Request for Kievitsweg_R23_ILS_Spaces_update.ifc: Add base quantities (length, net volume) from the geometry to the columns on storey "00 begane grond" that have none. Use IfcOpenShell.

First a look at what the model holds.

```python
import ifcopenshell
import ifcopenshell.util.element
import ifcopenshell.util.unit

model = ifcopenshell.open("Kievitsweg_R23_ILS_Spaces_update.ifc")
print(model.schema)
for unit_type in ("LENGTHUNIT", "AREAUNIT", "VOLUMEUNIT"):
    print(unit_type, ifcopenshell.util.unit.calculate_unit_scale(model, unit_type))
storey = next(s for s in model.by_type("IfcBuildingStorey") if s.Name == "00 begane grond")
columns = [e for e in ifcopenshell.util.element.get_decomposition(storey) if e.is_a("IfcColumn")]
for e in sorted(columns, key=lambda e: e.id()):
    print(e.id(), e.is_a(), e.Name, list(ifcopenshell.util.element.get_psets(e, qtos_only=True)), sep=" | ")
```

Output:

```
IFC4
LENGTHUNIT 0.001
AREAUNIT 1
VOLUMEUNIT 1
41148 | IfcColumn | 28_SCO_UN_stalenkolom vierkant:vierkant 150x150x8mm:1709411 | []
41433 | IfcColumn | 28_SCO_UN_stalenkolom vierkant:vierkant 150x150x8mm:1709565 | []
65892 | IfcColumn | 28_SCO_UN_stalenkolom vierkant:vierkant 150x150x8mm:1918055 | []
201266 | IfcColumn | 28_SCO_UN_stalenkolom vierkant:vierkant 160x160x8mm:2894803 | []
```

```python
import ifcopenshell
import ifcopenshell.api.pset
import ifcopenshell.geom
import ifcopenshell.util.element
import ifcopenshell.util.shape
import ifcopenshell.util.unit

model = ifcopenshell.open("Kievitsweg_R23_ILS_Spaces_update.ifc")
unit_scale = ifcopenshell.util.unit.calculate_unit_scale(model)
volume_scale = ifcopenshell.util.unit.calculate_unit_scale(model, "VOLUMEUNIT")
settings = ifcopenshell.geom.settings()

storey = next(s for s in model.by_type("IfcBuildingStorey") if s.Name == "00 begane grond")
columns = [e for e in ifcopenshell.util.element.get_decomposition(storey) if e.is_a("IfcColumn")]

for e in sorted(columns, key=lambda e: e.id()):
    if ifcopenshell.util.element.get_psets(e, qtos_only=True, should_inherit=False):
        continue
    # Geometry comes back in metres, in the element's own axes.
    shape = ifcopenshell.geom.create_shape(settings, e)
    values = {
        "Length": ifcopenshell.util.shape.get_z(shape.geometry) / unit_scale,
        "NetVolume": ifcopenshell.util.shape.get_volume(shape.geometry) / volume_scale,
    }
    qto = ifcopenshell.api.pset.add_qto(model, product=e, name="Qto_ColumnBaseQuantities")
    ifcopenshell.api.pset.edit_qto(model, qto=qto, properties=values)
    print(e.id(), {k: round(v, 3) for k, v in values.items()})

model.write("Kievitsweg_R23_ILS_Spaces_update_updated.ifc")
```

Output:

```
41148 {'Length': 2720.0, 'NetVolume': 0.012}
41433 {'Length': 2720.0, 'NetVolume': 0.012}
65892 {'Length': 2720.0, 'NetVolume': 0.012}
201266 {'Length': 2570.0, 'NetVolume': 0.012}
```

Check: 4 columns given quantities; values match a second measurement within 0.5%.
